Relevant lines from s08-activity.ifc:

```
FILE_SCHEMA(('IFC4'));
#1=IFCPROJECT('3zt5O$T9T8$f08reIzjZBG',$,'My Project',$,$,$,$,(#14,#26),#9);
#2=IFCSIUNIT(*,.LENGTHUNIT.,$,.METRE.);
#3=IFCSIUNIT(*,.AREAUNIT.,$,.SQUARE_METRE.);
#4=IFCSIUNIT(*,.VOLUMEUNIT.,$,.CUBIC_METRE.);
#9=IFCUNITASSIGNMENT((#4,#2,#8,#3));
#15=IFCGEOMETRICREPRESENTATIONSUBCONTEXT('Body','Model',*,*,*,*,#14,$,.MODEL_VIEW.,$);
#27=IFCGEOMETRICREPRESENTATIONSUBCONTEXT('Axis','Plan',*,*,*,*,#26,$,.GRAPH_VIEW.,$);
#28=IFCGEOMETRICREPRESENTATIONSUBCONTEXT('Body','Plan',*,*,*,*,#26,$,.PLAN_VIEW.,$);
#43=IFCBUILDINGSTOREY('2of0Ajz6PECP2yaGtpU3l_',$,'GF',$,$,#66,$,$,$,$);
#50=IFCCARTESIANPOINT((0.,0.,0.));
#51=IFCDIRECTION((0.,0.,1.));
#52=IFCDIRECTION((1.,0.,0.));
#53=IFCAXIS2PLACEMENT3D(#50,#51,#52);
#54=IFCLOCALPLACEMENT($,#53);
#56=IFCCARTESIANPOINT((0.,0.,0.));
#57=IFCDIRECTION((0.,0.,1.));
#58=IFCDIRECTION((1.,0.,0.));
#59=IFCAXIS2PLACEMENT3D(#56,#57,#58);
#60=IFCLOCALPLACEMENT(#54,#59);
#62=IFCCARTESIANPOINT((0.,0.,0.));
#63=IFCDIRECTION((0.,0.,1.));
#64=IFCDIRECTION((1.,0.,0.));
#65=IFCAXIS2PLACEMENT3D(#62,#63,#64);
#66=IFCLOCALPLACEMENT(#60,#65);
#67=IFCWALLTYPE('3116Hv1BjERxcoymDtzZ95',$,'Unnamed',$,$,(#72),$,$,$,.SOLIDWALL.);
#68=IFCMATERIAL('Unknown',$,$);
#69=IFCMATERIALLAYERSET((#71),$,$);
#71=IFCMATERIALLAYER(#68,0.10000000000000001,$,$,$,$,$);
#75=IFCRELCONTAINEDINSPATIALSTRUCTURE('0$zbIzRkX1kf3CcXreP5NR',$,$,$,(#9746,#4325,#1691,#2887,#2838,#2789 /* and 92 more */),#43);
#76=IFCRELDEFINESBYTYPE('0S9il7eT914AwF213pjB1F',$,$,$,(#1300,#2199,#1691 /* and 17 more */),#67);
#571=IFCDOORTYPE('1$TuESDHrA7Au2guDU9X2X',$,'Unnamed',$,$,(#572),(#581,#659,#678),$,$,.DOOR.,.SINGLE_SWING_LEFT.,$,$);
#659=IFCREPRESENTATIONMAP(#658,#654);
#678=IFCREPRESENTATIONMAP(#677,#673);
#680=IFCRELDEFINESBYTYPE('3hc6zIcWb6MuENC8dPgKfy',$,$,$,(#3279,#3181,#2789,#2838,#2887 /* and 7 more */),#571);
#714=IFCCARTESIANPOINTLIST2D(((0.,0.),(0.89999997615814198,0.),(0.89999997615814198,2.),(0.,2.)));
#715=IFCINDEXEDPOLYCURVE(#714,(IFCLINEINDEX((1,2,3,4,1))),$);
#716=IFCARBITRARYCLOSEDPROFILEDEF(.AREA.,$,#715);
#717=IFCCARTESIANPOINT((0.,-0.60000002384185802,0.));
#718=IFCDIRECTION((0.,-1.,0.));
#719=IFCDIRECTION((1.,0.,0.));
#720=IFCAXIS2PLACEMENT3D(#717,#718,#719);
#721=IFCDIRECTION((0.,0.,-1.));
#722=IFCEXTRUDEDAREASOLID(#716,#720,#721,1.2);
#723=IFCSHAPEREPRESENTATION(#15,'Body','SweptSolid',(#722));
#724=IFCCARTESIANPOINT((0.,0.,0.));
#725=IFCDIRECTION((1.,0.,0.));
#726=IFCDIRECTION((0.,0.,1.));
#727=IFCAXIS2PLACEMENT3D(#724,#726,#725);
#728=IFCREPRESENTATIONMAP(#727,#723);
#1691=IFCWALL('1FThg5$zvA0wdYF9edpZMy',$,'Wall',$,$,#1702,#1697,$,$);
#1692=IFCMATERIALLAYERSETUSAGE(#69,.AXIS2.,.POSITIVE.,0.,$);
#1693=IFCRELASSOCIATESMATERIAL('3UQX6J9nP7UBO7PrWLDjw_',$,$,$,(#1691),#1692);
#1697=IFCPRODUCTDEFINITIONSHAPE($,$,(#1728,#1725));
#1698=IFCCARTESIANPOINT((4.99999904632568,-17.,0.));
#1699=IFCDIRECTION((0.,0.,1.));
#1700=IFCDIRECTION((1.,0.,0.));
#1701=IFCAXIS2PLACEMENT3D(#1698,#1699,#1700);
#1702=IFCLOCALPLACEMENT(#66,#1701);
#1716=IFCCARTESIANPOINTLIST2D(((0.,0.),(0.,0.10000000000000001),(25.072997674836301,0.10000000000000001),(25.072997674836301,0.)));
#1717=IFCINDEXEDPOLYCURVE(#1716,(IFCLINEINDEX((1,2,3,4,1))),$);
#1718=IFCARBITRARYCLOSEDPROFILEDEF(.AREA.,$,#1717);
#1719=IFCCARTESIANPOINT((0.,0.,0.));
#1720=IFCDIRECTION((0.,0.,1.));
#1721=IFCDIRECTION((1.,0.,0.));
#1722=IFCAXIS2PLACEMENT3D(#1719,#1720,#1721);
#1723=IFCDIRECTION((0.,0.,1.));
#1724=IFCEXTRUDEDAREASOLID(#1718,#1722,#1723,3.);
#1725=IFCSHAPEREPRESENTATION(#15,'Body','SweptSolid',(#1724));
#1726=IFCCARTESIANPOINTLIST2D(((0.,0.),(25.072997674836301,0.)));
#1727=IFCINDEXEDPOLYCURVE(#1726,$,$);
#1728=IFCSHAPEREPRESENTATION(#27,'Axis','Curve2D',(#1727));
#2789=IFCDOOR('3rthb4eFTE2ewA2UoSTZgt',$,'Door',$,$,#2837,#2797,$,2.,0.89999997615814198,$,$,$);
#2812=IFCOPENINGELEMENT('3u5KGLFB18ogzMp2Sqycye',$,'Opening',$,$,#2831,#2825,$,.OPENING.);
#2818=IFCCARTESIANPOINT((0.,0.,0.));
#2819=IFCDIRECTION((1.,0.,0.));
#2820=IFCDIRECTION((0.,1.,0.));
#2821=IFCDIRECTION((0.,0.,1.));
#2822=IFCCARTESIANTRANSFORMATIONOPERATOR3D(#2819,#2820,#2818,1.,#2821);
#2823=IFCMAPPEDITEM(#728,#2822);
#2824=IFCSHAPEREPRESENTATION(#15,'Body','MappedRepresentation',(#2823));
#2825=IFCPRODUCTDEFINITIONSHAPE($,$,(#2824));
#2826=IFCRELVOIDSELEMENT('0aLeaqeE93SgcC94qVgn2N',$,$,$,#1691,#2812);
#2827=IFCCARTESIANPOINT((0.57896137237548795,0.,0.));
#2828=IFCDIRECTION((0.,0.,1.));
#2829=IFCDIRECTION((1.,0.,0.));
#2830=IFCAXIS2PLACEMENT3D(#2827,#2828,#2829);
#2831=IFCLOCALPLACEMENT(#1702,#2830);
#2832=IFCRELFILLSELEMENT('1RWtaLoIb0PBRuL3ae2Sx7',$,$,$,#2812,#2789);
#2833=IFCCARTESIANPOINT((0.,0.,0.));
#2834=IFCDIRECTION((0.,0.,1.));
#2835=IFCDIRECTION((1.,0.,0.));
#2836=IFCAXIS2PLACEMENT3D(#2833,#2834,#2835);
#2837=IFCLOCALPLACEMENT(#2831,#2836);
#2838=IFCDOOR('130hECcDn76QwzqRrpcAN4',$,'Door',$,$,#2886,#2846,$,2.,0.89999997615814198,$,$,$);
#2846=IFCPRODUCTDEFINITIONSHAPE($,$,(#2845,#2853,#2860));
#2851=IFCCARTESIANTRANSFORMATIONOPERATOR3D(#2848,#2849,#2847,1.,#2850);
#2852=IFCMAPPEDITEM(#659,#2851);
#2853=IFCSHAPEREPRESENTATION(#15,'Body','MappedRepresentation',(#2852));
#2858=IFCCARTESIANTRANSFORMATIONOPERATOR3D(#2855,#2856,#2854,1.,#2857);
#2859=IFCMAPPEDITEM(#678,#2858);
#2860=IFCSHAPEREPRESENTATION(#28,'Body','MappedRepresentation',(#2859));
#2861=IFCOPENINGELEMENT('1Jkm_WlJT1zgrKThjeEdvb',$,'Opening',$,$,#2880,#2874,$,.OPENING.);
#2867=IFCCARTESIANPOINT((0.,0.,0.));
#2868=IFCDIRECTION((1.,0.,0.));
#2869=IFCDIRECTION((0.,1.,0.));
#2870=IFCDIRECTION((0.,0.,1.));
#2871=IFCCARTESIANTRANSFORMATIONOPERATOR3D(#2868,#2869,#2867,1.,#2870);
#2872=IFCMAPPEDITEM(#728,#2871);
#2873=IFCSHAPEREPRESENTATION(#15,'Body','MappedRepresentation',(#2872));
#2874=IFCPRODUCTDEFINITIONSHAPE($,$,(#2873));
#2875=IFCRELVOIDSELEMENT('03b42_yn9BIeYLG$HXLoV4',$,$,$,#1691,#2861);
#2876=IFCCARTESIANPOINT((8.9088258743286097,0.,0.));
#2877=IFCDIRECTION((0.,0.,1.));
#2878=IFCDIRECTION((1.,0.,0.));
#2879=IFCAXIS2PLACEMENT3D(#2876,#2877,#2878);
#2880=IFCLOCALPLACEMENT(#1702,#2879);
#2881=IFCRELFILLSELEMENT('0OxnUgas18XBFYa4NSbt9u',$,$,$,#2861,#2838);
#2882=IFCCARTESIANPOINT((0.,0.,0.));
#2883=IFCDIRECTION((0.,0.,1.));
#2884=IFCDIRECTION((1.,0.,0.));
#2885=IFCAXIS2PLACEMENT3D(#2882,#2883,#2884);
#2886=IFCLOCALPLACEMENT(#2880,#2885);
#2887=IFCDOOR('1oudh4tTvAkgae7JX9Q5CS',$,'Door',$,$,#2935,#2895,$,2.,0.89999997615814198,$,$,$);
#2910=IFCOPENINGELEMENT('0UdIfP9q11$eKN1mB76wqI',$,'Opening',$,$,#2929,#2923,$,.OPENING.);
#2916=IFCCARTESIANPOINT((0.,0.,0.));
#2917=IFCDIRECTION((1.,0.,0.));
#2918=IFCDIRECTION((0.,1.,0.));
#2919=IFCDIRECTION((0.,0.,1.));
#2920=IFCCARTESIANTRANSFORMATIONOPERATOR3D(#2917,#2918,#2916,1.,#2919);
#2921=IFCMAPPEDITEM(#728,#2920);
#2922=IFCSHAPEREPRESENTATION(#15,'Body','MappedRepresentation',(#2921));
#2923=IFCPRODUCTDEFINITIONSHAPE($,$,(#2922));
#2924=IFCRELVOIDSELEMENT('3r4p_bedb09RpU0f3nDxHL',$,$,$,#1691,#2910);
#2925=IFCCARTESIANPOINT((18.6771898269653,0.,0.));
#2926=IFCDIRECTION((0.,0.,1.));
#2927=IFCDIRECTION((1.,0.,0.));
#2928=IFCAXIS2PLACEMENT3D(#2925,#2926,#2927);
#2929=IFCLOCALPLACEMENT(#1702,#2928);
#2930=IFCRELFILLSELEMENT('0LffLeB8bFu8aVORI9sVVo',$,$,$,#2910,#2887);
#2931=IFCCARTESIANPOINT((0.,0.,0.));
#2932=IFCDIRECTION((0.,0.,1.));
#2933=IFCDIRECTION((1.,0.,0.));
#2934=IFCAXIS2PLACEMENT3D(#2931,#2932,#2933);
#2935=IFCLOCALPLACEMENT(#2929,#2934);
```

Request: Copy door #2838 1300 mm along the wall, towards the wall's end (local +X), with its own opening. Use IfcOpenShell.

```python
import ifcopenshell
import ifcopenshell.api.feature
import ifcopenshell.api.geometry
import ifcopenshell.api.root
import ifcopenshell.geom
import ifcopenshell.util.element
import ifcopenshell.util.placement
import ifcopenshell.util.shape

model = ifcopenshell.open("s08-activity.ifc")
settings = ifcopenshell.geom.settings()


def volume(element):
    """Net volume in cubic metres, openings subtracted."""
    shape = ifcopenshell.geom.create_shape(settings, element)
    return ifcopenshell.util.shape.get_volume(shape.geometry)


door = model.by_id(2838)
opening = door.FillsVoids[0].RelatingOpeningElement
wall = opening.VoidsElements[0].RelatingBuildingElement
before = volume(wall)
shift = ifcopenshell.util.placement.get_local_placement(wall.ObjectPlacement)[:3, 0] * 1.3

# copy_class copies the void relationship, type, container and properties, but no geometry.
new_opening = ifcopenshell.api.root.copy_class(model, product=opening)
new_opening.Representation = ifcopenshell.util.element.copy_deep(
    model, opening.Representation, exclude=["IfcGeometricRepresentationContext", "IfcRepresentationMap"]
)
new_door = ifcopenshell.api.root.copy_class(model, product=door)
new_door.Representation = ifcopenshell.util.element.copy_deep(
    model, door.Representation, exclude=["IfcGeometricRepresentationContext", "IfcRepresentationMap"]
)
ifcopenshell.api.feature.add_filling(model, opening=new_opening, element=new_door)

for old, new in ((opening, new_opening), (door, new_door)):
    matrix = ifcopenshell.util.placement.get_local_placement(old.ObjectPlacement)
    matrix[:3, 3] += shift
    ifcopenshell.api.geometry.edit_object_placement(model, product=new, matrix=matrix, is_si=False)

after = volume(wall)

print(f"wall volume {before:.3f} -> {after:.3f} m3")

model.write("s08-activity_edited.ifc")
```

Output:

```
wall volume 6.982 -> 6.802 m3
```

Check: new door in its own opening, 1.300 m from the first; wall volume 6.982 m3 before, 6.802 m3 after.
